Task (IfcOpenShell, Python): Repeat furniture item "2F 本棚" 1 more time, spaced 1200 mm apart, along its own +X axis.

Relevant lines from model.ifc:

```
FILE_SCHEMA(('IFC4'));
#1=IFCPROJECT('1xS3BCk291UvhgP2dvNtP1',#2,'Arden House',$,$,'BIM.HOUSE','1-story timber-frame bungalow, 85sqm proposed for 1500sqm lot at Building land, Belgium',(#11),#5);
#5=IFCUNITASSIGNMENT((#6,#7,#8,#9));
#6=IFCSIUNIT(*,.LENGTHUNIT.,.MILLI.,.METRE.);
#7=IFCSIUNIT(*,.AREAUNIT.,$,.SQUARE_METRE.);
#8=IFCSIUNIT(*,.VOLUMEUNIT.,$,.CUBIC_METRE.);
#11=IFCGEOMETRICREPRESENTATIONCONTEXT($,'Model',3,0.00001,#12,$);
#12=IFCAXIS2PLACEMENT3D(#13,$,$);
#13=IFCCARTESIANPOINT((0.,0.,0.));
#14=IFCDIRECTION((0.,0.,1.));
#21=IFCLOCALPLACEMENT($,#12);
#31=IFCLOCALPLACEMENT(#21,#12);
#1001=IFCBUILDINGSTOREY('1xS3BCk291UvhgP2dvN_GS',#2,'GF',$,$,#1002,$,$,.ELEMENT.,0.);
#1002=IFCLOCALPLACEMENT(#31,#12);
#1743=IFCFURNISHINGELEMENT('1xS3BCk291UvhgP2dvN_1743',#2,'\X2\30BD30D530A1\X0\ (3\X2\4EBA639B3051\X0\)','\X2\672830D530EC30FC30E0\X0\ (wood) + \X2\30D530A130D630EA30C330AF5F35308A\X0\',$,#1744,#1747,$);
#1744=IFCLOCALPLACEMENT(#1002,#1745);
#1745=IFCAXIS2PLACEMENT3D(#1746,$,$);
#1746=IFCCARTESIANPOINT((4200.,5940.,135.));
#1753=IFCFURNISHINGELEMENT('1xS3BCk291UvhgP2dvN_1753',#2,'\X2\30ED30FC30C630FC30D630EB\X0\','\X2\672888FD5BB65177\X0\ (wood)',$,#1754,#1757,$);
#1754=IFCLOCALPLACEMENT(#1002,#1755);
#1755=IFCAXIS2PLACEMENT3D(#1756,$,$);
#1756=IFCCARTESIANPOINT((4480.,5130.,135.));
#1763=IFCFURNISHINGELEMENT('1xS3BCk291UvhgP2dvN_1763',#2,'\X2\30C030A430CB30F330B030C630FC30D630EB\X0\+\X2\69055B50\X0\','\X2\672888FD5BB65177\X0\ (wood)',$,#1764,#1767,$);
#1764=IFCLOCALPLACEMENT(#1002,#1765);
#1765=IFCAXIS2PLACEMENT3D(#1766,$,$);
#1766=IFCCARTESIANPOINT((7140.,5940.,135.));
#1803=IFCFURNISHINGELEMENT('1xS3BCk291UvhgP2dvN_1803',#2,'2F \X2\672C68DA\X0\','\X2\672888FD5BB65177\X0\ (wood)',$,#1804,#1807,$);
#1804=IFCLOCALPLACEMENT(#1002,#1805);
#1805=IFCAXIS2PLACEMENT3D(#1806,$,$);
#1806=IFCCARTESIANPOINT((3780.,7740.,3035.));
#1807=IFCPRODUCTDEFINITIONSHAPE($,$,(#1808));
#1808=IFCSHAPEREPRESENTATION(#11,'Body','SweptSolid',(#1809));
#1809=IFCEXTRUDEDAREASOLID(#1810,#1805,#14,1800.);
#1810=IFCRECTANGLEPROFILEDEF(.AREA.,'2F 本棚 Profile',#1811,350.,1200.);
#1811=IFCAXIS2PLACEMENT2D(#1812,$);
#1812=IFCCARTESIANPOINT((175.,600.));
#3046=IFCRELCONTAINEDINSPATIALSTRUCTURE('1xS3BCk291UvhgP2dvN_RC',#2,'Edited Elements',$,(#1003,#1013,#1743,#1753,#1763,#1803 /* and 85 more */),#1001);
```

```python
import ifcopenshell
import ifcopenshell.api.geometry
import ifcopenshell.api.root
import ifcopenshell.util.element
import ifcopenshell.util.placement

model = ifcopenshell.open("model.ifc")


def reuse_history(source, copy):
    """copy_class also copies each property set's owner history, people and application; keep the originals."""
    for rel in copy.IsDefinedBy:
        if rel.is_a("IfcRelDefinesByProperties") and (history := rel.RelatingPropertyDefinition.OwnerHistory):
            rel.RelatingPropertyDefinition.OwnerHistory = source.OwnerHistory
            ifcopenshell.util.element.remove_deep2(model, history)


source = model.by_id(1803)
base = ifcopenshell.util.placement.get_local_placement(source.ObjectPlacement)
step = base[:3, 0] * 1200.0

for i in range(1, 2):
    copy = ifcopenshell.api.root.copy_class(model, product=source)
    copy.Representation = ifcopenshell.util.element.copy_deep(
        model, source.Representation, exclude=["IfcGeometricRepresentationContext", "IfcRepresentationMap"]
    )
    reuse_history(source, copy)
    matrix = base.copy()
    matrix[:3, 3] += i * step
    print("added at", matrix[:3, 3].round(3) + 0.0)
    ifcopenshell.api.geometry.edit_object_placement(model, product=copy, matrix=matrix, is_si=False)

model.write("model_updated.ifc")
```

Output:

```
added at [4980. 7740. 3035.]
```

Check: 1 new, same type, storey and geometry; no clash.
